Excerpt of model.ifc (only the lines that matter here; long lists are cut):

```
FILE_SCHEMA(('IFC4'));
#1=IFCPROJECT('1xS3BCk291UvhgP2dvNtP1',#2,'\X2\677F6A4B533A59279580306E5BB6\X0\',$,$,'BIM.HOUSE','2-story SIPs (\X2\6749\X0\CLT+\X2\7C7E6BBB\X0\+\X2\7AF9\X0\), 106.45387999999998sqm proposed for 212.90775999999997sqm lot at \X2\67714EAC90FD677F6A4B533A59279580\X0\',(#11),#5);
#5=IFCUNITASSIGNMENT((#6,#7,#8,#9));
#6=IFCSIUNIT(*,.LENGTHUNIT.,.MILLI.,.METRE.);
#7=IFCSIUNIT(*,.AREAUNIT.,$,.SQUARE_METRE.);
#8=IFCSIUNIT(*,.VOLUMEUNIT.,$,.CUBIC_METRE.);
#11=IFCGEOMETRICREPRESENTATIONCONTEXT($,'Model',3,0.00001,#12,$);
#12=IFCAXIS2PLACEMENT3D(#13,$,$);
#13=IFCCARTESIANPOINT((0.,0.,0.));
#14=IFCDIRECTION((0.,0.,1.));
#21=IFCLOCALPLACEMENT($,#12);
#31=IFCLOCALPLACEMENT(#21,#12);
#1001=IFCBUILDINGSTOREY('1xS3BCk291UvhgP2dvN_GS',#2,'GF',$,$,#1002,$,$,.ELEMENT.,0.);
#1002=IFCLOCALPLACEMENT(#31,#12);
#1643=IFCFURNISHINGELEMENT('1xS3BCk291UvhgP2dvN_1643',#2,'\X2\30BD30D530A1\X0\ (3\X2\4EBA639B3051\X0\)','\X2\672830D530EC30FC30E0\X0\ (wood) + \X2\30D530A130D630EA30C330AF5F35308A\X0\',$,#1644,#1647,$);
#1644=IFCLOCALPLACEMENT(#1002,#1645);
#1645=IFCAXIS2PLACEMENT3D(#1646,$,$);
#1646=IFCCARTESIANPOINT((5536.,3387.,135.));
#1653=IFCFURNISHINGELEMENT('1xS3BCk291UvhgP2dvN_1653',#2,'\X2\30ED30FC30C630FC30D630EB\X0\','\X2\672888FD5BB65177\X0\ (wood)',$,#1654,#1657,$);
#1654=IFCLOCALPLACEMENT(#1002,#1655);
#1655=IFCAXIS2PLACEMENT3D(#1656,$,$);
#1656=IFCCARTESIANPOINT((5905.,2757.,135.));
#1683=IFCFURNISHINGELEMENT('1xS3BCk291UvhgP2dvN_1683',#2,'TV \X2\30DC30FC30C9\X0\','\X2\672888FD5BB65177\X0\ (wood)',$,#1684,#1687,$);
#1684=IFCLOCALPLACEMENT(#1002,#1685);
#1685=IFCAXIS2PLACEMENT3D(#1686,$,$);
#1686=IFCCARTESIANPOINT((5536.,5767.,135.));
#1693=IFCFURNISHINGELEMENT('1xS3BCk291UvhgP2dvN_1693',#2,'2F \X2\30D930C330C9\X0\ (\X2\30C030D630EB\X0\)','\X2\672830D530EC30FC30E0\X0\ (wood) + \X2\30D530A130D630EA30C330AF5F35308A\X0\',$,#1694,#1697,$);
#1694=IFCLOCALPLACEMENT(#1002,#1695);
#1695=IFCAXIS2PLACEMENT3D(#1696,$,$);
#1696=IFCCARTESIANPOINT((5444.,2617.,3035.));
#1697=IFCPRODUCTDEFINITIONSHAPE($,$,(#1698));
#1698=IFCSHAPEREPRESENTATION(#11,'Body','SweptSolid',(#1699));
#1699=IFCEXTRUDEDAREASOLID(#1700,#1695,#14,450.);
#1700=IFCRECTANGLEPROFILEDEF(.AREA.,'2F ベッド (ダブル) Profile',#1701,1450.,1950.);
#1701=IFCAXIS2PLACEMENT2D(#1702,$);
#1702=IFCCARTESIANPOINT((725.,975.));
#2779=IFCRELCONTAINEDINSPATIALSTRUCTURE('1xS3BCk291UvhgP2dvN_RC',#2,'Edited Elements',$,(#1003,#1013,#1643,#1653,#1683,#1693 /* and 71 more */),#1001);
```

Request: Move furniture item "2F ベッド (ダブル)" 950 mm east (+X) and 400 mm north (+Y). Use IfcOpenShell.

```python
import ifcopenshell
import ifcopenshell.api.geometry
import ifcopenshell.util.placement

model = ifcopenshell.open("model.ifc")

item = model.by_id(1693)
matrix = ifcopenshell.util.placement.get_local_placement(item.ObjectPlacement)
matrix[0, 3] += 950.0
matrix[1, 3] += 400.0
ifcopenshell.api.geometry.edit_object_placement(model, product=item, matrix=matrix, is_si=False)

print(ifcopenshell.util.placement.get_local_placement(item.ObjectPlacement).round(3) + 0.0)

model.write("model_edited.ifc")
```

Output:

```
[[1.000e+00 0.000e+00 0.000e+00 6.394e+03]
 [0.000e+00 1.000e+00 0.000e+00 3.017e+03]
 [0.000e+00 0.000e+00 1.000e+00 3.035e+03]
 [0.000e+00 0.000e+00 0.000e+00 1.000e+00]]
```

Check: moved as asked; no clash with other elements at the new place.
